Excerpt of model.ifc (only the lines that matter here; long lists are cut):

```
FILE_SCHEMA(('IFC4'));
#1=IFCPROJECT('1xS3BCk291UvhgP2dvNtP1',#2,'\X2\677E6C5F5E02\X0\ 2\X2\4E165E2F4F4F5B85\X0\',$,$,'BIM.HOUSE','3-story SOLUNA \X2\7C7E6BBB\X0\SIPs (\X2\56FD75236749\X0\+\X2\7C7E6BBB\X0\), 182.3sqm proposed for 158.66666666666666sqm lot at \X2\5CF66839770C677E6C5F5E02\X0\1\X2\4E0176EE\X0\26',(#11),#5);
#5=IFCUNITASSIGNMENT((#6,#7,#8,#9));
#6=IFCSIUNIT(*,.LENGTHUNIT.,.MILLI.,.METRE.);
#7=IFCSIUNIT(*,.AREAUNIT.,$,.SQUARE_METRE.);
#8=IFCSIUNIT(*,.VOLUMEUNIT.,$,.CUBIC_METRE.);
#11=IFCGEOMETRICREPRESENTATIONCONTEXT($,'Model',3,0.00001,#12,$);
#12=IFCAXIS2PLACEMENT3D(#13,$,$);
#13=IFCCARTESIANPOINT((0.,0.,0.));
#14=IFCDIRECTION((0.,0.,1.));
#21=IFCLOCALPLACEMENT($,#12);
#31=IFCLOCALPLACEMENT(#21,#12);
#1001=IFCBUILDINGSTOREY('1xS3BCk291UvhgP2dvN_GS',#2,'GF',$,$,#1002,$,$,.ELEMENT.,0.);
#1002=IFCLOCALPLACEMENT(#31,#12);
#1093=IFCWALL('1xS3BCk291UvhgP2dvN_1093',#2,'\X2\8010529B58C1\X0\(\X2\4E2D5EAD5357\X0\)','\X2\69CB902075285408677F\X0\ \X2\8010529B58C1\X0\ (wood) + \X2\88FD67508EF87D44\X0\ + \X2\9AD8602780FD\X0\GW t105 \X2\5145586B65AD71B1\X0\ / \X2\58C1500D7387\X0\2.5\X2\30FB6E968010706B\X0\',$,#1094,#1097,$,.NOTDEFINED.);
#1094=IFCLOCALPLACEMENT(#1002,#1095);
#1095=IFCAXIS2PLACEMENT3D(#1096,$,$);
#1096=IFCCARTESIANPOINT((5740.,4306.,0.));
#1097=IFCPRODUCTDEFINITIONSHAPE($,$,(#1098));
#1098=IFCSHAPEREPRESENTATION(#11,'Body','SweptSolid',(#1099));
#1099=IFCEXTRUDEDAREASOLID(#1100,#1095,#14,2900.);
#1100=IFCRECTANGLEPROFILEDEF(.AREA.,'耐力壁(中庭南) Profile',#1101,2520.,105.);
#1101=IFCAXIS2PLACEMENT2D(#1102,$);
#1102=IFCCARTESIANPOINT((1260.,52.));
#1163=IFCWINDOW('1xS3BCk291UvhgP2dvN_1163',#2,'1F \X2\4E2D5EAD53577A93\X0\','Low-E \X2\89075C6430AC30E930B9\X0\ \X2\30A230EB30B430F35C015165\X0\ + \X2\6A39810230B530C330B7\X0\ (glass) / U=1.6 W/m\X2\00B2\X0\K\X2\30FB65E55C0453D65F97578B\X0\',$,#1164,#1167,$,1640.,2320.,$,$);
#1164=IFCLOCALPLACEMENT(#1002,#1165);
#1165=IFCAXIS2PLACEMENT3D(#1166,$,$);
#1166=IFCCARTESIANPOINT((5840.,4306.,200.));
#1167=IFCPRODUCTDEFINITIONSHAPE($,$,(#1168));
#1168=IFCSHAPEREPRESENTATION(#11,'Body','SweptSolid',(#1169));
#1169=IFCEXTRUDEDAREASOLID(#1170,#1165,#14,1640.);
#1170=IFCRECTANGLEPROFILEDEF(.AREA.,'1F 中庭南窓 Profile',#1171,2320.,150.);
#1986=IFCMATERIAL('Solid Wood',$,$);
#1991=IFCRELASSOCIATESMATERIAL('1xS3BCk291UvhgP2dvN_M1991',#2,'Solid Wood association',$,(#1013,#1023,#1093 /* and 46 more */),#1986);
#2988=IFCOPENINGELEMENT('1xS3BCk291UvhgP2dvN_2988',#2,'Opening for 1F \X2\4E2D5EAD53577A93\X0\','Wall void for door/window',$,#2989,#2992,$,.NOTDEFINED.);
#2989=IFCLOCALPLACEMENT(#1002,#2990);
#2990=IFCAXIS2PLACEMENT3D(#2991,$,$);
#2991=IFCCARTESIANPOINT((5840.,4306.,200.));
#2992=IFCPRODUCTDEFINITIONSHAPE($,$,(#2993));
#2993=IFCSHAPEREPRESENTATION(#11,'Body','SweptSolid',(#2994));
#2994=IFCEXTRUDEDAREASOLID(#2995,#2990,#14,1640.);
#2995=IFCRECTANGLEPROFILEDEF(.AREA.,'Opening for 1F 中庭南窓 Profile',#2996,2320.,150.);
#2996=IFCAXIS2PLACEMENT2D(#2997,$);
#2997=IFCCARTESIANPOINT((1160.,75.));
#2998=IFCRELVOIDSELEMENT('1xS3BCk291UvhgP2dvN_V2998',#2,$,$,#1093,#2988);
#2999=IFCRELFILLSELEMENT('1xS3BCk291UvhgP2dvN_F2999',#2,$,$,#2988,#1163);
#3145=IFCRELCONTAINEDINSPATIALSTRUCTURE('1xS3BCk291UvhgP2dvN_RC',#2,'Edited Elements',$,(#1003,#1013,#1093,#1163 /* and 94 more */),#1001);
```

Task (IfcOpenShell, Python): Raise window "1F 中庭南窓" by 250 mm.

```python
import numpy as np
import ifcopenshell
import ifcopenshell.api.geometry
import ifcopenshell.util.placement
import ifcopenshell.util.unit

model = ifcopenshell.open("model.ifc")
unit_scale = ifcopenshell.util.unit.calculate_unit_scale(model)

window = model.by_guid("1xS3BCk291UvhgP2dvN_1163")
opening = window.FillsVoids[0].RelatingOpeningElement
dz = 0.25 / unit_scale

shift = np.array([0.0, 0.0, dz])
# The window is not placed relative to its opening, so move both.
for product in (opening, window):
    matrix = ifcopenshell.util.placement.get_local_placement(product.ObjectPlacement)
    matrix[:3, 3] += shift
    ifcopenshell.api.geometry.edit_object_placement(model, product=product, matrix=matrix, is_si=False)

print(f"moved by {dz * unit_scale:+.3f} m")

model.write("model_rev.ifc")
```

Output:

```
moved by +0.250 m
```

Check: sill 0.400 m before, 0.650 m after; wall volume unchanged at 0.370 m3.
